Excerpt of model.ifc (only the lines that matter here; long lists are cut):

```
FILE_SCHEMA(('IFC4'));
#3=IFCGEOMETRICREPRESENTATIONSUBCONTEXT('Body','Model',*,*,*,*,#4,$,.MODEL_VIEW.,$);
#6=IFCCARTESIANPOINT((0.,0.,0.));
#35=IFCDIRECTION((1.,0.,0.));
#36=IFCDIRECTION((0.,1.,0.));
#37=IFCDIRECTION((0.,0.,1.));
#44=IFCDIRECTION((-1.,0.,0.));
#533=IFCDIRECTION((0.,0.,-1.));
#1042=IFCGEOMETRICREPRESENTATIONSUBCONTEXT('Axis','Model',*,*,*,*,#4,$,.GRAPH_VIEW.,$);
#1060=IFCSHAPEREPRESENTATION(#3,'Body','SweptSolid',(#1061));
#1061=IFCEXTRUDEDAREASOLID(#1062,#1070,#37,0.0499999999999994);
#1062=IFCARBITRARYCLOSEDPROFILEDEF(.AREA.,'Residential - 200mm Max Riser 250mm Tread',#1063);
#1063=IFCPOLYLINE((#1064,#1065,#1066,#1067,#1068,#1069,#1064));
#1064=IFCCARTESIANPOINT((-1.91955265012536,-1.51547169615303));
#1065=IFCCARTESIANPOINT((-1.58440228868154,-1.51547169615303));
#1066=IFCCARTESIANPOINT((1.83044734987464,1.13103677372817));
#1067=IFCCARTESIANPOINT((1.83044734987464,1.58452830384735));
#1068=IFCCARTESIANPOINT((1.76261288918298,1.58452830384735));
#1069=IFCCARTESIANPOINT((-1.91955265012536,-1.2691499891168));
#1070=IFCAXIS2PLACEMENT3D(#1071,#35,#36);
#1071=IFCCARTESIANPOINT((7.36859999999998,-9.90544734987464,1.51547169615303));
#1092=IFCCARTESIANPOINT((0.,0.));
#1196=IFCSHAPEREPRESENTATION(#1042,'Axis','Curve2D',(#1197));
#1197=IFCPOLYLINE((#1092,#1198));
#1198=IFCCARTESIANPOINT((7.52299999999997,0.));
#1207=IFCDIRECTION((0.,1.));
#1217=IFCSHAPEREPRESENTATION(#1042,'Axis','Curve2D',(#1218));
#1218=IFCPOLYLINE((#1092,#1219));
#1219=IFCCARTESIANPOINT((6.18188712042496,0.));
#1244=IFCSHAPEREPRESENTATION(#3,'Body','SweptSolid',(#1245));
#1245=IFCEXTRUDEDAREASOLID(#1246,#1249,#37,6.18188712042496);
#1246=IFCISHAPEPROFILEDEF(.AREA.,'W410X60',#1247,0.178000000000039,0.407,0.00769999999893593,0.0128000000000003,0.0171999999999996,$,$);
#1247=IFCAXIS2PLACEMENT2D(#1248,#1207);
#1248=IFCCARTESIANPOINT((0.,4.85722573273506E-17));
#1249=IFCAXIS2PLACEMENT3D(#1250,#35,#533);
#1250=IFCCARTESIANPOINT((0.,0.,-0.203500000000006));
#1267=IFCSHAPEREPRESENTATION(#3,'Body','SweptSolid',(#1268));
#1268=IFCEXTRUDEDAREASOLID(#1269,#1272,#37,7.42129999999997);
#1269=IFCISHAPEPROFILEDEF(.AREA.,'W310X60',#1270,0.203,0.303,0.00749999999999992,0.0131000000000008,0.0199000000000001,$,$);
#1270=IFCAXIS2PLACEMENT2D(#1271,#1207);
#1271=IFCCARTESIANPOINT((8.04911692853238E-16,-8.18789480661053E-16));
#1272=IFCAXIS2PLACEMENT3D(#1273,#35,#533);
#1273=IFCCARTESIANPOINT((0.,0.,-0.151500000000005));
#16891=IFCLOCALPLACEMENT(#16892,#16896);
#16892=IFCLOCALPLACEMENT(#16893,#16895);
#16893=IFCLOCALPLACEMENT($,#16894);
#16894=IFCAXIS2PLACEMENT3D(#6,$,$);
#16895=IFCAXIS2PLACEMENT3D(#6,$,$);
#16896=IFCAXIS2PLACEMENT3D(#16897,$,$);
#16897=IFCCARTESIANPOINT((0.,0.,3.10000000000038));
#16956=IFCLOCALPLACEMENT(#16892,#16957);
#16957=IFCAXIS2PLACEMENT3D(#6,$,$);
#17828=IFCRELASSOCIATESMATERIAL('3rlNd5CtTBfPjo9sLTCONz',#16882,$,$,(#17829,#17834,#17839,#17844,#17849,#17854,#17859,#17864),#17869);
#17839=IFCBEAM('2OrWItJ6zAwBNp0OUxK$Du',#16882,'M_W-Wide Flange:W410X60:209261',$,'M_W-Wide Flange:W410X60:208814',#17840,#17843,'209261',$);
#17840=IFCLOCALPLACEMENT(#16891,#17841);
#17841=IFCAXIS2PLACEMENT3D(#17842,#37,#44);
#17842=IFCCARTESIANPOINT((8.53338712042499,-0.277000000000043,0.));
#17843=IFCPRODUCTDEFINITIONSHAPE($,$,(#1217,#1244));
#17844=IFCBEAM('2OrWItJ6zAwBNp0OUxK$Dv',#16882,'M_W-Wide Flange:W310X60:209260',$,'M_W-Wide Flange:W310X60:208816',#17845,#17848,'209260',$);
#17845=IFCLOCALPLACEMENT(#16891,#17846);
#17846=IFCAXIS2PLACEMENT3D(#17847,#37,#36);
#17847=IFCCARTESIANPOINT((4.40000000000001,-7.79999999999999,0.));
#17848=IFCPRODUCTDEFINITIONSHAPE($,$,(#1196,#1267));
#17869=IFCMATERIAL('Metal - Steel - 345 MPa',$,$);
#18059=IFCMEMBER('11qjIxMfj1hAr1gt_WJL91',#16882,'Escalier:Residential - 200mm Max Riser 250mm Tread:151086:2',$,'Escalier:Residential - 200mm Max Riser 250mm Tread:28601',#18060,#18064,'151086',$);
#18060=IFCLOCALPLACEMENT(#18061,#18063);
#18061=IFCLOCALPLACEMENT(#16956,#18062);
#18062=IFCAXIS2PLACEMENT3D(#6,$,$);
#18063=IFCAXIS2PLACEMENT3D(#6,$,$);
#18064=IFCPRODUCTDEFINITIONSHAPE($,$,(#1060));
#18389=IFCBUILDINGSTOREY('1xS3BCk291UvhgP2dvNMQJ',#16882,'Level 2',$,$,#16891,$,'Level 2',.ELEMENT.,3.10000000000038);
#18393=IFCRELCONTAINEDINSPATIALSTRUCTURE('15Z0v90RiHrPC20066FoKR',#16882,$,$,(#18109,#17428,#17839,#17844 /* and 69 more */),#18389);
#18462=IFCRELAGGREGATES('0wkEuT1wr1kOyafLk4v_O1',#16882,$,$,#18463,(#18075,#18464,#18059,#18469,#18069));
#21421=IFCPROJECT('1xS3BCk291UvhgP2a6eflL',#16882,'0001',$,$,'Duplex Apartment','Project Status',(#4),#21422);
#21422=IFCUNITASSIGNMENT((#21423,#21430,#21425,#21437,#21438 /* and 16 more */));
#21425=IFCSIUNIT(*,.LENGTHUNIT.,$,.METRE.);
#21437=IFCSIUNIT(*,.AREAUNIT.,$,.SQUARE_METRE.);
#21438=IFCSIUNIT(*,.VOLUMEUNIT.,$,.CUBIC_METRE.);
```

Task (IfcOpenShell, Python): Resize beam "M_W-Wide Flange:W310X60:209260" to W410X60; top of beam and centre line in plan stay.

```python
import ifcopenshell
import ifcopenshell.util.element
import ifcopenshell.util.representation

model = ifcopenshell.open("model.ifc")

member = model.by_guid("2OrWItJ6zAwBNp0OUxK$Dv")
source = next(p for p in model.by_type("IfcIShapeProfileDef") if p.ProfileName == "W410X60")

body = ifcopenshell.util.representation.get_representation(member, "Model", "Body")
solid = body.Items[0]
old_profile = solid.SweptArea

# Copy the section's sizes but keep this member's own profile position.
profile = ifcopenshell.util.element.copy(model, source)
# Profiles are centred, so shift by half the change in depth to hold the top.
shift = (old_profile.OverallDepth - profile.OverallDepth) / 2
x, y = old_profile.Position.Location.Coordinates
up = (-1.0, 0.0)  # upwards, in the solid's own plane
location = model.createIfcCartesianPoint((x + up[0] * shift, y + up[1] * shift))
profile.Position = model.createIfcAxis2Placement2D(location, old_profile.Position.RefDirection)
solid.SweptArea = profile
if not model.get_total_inverses(old_profile):
    ifcopenshell.util.element.remove_deep2(model, old_profile)
member.Name = member.Name.replace("W310X60", "W410X60")
member.ObjectType = member.ObjectType.replace("W310X60", "W410X60")

print(solid.SweptArea)

model.write("model-out.ifc")
```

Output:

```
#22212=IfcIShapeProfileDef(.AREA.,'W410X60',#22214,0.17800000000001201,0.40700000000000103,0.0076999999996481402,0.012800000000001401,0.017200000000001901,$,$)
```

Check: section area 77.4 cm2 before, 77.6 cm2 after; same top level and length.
